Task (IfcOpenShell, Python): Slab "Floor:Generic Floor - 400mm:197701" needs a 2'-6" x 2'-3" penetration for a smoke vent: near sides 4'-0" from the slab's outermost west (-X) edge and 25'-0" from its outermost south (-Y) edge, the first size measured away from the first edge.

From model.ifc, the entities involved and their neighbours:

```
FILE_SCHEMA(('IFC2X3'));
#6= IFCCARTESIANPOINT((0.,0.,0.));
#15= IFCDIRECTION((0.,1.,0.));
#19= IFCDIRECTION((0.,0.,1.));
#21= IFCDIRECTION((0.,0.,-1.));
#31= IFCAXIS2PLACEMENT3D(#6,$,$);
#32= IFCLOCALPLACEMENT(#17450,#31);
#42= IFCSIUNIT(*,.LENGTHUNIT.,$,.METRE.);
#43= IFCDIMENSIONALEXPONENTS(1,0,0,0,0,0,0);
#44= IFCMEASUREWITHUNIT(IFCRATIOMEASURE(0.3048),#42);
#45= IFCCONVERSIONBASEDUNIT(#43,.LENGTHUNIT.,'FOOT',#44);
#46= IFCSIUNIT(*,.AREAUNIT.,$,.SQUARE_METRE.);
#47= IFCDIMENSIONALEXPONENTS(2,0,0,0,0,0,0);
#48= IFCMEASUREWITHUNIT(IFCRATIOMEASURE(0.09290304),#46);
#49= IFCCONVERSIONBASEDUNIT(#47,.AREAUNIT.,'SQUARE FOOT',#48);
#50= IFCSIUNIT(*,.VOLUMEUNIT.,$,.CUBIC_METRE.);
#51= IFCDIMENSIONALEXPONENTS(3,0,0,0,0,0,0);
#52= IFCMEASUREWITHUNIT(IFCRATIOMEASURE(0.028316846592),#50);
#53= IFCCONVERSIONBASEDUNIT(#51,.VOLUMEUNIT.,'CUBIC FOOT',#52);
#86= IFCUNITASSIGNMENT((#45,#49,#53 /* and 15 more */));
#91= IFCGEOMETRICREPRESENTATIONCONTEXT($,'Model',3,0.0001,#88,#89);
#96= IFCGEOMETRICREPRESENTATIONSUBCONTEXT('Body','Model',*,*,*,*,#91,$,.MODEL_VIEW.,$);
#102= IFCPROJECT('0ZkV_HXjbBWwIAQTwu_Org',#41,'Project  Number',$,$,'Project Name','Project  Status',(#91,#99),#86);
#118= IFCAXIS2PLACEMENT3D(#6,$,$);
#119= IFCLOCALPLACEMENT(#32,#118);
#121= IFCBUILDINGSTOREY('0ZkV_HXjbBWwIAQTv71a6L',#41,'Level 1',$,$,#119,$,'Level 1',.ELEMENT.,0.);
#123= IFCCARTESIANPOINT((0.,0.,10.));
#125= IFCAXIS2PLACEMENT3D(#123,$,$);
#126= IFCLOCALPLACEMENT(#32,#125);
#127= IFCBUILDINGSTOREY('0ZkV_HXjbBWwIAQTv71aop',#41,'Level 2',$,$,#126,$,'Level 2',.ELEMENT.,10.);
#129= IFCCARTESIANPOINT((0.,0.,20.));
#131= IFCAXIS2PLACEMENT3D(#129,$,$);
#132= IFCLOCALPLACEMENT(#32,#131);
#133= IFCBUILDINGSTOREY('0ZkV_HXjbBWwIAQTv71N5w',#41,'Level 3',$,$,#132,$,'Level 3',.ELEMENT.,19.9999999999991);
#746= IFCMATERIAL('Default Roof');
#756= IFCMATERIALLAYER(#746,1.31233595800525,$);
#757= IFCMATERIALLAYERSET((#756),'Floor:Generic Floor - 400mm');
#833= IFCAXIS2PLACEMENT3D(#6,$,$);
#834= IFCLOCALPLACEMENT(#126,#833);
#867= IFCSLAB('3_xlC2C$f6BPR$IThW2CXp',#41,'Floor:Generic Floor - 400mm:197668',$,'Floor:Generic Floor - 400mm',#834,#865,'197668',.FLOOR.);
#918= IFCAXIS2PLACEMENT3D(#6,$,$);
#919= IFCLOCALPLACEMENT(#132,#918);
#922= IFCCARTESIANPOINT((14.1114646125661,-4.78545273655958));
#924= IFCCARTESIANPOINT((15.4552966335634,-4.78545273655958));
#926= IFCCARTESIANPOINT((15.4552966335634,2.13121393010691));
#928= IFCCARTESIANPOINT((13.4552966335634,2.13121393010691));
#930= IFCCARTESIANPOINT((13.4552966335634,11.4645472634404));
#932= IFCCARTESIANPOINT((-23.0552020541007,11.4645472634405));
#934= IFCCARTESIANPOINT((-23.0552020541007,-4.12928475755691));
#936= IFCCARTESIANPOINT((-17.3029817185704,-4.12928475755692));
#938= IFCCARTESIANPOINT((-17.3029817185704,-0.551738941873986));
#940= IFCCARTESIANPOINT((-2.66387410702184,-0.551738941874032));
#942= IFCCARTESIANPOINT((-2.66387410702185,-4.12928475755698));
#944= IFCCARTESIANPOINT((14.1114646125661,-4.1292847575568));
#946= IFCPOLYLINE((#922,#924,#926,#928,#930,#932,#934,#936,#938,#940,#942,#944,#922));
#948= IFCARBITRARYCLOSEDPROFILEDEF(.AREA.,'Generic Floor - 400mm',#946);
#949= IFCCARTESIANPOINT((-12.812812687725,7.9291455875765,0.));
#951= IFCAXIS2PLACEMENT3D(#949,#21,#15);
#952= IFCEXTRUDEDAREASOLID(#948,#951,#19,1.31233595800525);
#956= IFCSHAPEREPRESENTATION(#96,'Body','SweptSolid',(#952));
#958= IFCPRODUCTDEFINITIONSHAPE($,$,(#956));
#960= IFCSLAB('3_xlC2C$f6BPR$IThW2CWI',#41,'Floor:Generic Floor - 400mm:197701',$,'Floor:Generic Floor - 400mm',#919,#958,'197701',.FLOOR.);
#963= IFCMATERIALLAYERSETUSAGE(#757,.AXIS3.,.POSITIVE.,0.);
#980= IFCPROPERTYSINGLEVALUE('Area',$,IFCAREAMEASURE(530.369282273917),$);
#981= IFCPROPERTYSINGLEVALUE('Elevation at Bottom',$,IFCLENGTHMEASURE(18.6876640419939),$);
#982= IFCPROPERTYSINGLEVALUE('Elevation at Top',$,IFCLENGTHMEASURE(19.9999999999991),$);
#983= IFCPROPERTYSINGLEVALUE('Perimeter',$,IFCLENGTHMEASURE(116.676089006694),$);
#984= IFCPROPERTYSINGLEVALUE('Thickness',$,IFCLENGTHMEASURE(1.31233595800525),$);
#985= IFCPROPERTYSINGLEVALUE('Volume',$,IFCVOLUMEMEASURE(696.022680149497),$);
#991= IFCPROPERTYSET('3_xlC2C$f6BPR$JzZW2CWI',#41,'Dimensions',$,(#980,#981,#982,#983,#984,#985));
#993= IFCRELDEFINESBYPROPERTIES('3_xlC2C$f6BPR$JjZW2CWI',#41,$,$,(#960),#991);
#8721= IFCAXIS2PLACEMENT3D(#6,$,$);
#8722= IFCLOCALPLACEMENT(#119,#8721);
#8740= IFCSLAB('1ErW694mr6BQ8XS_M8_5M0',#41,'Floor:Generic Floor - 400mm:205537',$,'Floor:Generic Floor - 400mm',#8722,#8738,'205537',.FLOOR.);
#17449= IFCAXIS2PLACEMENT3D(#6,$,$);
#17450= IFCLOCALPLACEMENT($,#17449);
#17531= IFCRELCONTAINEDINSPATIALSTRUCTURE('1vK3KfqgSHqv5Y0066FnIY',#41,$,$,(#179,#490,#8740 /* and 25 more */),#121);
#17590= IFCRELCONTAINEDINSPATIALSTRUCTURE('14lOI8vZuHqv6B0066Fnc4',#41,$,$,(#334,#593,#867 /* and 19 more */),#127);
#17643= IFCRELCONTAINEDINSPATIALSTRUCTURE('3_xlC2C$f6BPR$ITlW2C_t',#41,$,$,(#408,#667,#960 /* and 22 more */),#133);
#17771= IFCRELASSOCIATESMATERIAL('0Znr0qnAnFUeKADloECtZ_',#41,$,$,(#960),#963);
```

```python
import numpy as np
import ifcopenshell
import ifcopenshell.api.feature
import ifcopenshell.api.geometry
import ifcopenshell.api.pset
import ifcopenshell.api.root
import ifcopenshell.geom
import ifcopenshell.util.element
import ifcopenshell.util.placement
import ifcopenshell.util.representation
import ifcopenshell.util.shape
import ifcopenshell.util.unit

model = ifcopenshell.open("model.ifc")
unit_scale = ifcopenshell.util.unit.calculate_unit_scale(model)
area_scale = ifcopenshell.util.unit.calculate_unit_scale(model, "AREAUNIT")
volume_scale = ifcopenshell.util.unit.calculate_unit_scale(model, "VOLUMEUNIT")
settings = ifcopenshell.geom.settings()


def volume(element):
    """Net volume in cubic metres, openings subtracted."""
    shape = ifcopenshell.geom.create_shape(settings, element)
    return ifcopenshell.util.shape.get_volume(shape.geometry)


slab = model.by_guid("3_xlC2C$f6BPR$IThW2CWI")
before = volume(slab)

# Extent in the slab's own axes, in metres. The edges named are its -X and -Y sides.
slab_shape = ifcopenshell.geom.create_shape(settings, slab)
vertices = ifcopenshell.util.shape.get_vertices(slab_shape.geometry)
x_min, y_min, bottom = vertices.min(axis=0)
top = vertices[:, 2].max()

opening = ifcopenshell.api.root.create_entity(model, ifc_class="IfcOpeningElement", name="Smoke vent opening")
context = ifcopenshell.util.representation.get_context(model, "Model", "Body", "MODEL_VIEW")
width, depth = 0.762, 0.6858
outline = [(0.0, 0.0), (width, 0.0), (width, depth), (0.0, depth), (0.0, 0.0)]
# Overshoot both faces by 50 mm so the cut is clean.
shape = ifcopenshell.api.geometry.add_slab_representation(
    model, context=context, depth=top - bottom + 0.1, polyline=outline
)
ifcopenshell.api.geometry.assign_representation(model, product=opening, representation=shape)

matrix = ifcopenshell.util.placement.get_local_placement(slab.ObjectPlacement)
matrix[:, 3] = matrix @ np.append(np.array([x_min + 1.2192, y_min + 7.62, bottom - 0.05]) / unit_scale, 1.0)
ifcopenshell.api.geometry.edit_object_placement(model, product=opening, matrix=matrix, is_si=False)
ifcopenshell.api.feature.add_feature(model, feature=opening, element=slab)

after = volume(slab)

# Update the slab's stored quantities.
pset = model.by_id(ifcopenshell.util.element.get_pset(slab, "Dimensions", should_inherit=False)["id"])
ifcopenshell.api.pset.edit_pset(model, pset=pset, properties={
    "Area": model.create_entity("IfcAreaMeasure", after / (top - bottom) / area_scale),
    "Volume": model.create_entity("IfcVolumeMeasure", after / volume_scale),
})

print(f"slab volume {before:.3f} -> {after:.3f} m3")

model.write("model-out.ifc")
```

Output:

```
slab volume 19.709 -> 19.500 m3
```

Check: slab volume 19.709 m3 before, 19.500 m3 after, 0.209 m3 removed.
